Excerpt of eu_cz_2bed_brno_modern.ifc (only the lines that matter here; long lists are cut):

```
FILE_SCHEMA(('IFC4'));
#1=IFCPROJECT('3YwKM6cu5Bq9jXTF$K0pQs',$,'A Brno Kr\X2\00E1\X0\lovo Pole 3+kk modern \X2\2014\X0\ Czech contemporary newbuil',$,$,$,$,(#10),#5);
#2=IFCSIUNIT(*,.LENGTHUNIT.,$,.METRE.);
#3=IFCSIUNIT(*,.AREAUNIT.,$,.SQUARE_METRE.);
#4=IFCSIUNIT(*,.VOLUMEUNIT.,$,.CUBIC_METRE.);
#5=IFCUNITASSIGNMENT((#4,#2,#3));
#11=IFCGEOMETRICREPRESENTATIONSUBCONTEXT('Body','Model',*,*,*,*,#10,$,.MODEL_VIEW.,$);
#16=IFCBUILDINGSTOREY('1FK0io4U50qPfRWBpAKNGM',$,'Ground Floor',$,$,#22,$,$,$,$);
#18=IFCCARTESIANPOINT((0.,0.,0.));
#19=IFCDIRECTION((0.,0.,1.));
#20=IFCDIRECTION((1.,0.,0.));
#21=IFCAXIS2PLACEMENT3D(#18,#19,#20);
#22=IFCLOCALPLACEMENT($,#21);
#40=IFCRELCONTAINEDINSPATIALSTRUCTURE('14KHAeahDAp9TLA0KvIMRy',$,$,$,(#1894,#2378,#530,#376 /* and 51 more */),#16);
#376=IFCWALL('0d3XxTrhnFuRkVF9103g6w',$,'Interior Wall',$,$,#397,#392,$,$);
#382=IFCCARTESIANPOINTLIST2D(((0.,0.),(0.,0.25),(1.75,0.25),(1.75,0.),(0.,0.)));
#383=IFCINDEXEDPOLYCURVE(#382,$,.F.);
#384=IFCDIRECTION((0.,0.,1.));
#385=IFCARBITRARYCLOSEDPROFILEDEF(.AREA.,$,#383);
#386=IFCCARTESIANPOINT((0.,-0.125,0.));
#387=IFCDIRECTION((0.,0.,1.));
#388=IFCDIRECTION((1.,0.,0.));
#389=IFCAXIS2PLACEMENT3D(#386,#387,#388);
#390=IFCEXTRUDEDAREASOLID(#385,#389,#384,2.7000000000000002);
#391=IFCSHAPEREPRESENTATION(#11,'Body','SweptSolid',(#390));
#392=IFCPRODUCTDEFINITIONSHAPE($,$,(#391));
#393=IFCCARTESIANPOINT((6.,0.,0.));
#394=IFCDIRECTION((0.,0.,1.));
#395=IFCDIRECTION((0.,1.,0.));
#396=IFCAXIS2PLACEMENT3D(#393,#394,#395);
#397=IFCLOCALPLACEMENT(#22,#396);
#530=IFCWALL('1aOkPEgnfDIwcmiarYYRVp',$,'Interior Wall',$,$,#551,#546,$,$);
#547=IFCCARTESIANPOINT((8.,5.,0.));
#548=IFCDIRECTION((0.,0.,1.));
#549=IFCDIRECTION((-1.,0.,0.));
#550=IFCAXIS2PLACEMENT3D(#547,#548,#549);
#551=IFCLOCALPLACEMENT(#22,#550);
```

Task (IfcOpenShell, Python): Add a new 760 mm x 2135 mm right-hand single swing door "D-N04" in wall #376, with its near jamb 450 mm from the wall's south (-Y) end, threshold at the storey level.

```python
import numpy as np
import ifcopenshell
import ifcopenshell.api.feature
import ifcopenshell.api.geometry
import ifcopenshell.api.root
import ifcopenshell.api.spatial
import ifcopenshell.geom
import ifcopenshell.util.element
import ifcopenshell.util.placement
import ifcopenshell.util.representation
import ifcopenshell.util.shape
import ifcopenshell.util.unit

model = ifcopenshell.open("eu_cz_2bed_brno_modern.ifc")
unit_scale = ifcopenshell.util.unit.calculate_unit_scale(model)
settings = ifcopenshell.geom.settings()


def volume(element):
    """Net volume in cubic metres, openings subtracted."""
    shape = ifcopenshell.geom.create_shape(settings, element)
    return ifcopenshell.util.shape.get_volume(shape.geometry)


wall = model.by_guid("0d3XxTrhnFuRkVF9103g6w")
storey = ifcopenshell.util.element.get_container(wall, ifc_class="IfcBuildingStorey")
context = ifcopenshell.util.representation.get_context(model, "Model", "Body", "MODEL_VIEW")
before = volume(wall)

width, height, from_end, sill = 0.76, 2.135, 0.45, 0.0  # metres

# The wall runs along its own X axis, and the end named is its -X end.
wall_shape = ifcopenshell.geom.create_shape(settings, wall)
x, y, z = ifcopenshell.util.shape.get_vertices(wall_shape.geometry).T
start = x.min() + from_end
face, thickness = float(y.min()), float(y.max() - y.min())
wall_matrix = ifcopenshell.util.placement.get_local_placement(wall.ObjectPlacement)
level = ifcopenshell.util.placement.get_local_placement(storey.ObjectPlacement)[2, 3]


def in_wall(x, y):
    """Placement at x, y metres in the wall's axes, at sill height."""
    matrix = wall_matrix.copy()
    matrix[:, 3] = wall_matrix @ np.array([x / unit_scale, y / unit_scale, 0.0, 1.0])
    matrix[2, 3] = level + sill / unit_scale
    return matrix


# Opening: a box that overshoots both wall faces by 50 mm.
opening = ifcopenshell.api.root.create_entity(model, ifc_class="IfcOpeningElement", predefined_type="OPENING")
box = ifcopenshell.api.geometry.add_wall_representation(
    model, context=context, length=width, height=height, thickness=thickness + 0.1
)
ifcopenshell.api.geometry.assign_representation(model, product=opening, representation=box)
ifcopenshell.api.geometry.edit_object_placement(model, product=opening, matrix=in_wall(start, face - 0.05), is_si=False)
ifcopenshell.api.feature.add_feature(model, feature=opening, element=wall)

door = ifcopenshell.api.root.create_entity(model, ifc_class="IfcDoor", name="D-N04", predefined_type="DOOR")
door.OverallWidth, door.OverallHeight = width / unit_scale, height / unit_scale
door.OperationType = "SINGLE_SWING_RIGHT"
body = ifcopenshell.api.geometry.add_door_representation(
    model,
    context=context,
    overall_width=door.OverallWidth,
    overall_height=door.OverallHeight,
    operation_type="SINGLE_SWING_RIGHT",
    lining_properties={"LiningDepth": thickness / unit_scale, "ThresholdDepth": thickness / unit_scale},
)
ifcopenshell.api.geometry.assign_representation(model, product=door, representation=body)
ifcopenshell.api.spatial.assign_container(model, products=[door], relating_structure=storey)
ifcopenshell.api.feature.add_filling(model, opening=opening, element=door)

# The lining spans the wall, so the door starts at the wall face.
ifcopenshell.api.geometry.edit_object_placement(model, product=door, matrix=in_wall(start, face), is_si=False)

after = volume(wall)

print(f"wall volume {before:.3f} -> {after:.3f} m3")

model.write("eu_cz_2bed_brno_modern_rev.ifc")
```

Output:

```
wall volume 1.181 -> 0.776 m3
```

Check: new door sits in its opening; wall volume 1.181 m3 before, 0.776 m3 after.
